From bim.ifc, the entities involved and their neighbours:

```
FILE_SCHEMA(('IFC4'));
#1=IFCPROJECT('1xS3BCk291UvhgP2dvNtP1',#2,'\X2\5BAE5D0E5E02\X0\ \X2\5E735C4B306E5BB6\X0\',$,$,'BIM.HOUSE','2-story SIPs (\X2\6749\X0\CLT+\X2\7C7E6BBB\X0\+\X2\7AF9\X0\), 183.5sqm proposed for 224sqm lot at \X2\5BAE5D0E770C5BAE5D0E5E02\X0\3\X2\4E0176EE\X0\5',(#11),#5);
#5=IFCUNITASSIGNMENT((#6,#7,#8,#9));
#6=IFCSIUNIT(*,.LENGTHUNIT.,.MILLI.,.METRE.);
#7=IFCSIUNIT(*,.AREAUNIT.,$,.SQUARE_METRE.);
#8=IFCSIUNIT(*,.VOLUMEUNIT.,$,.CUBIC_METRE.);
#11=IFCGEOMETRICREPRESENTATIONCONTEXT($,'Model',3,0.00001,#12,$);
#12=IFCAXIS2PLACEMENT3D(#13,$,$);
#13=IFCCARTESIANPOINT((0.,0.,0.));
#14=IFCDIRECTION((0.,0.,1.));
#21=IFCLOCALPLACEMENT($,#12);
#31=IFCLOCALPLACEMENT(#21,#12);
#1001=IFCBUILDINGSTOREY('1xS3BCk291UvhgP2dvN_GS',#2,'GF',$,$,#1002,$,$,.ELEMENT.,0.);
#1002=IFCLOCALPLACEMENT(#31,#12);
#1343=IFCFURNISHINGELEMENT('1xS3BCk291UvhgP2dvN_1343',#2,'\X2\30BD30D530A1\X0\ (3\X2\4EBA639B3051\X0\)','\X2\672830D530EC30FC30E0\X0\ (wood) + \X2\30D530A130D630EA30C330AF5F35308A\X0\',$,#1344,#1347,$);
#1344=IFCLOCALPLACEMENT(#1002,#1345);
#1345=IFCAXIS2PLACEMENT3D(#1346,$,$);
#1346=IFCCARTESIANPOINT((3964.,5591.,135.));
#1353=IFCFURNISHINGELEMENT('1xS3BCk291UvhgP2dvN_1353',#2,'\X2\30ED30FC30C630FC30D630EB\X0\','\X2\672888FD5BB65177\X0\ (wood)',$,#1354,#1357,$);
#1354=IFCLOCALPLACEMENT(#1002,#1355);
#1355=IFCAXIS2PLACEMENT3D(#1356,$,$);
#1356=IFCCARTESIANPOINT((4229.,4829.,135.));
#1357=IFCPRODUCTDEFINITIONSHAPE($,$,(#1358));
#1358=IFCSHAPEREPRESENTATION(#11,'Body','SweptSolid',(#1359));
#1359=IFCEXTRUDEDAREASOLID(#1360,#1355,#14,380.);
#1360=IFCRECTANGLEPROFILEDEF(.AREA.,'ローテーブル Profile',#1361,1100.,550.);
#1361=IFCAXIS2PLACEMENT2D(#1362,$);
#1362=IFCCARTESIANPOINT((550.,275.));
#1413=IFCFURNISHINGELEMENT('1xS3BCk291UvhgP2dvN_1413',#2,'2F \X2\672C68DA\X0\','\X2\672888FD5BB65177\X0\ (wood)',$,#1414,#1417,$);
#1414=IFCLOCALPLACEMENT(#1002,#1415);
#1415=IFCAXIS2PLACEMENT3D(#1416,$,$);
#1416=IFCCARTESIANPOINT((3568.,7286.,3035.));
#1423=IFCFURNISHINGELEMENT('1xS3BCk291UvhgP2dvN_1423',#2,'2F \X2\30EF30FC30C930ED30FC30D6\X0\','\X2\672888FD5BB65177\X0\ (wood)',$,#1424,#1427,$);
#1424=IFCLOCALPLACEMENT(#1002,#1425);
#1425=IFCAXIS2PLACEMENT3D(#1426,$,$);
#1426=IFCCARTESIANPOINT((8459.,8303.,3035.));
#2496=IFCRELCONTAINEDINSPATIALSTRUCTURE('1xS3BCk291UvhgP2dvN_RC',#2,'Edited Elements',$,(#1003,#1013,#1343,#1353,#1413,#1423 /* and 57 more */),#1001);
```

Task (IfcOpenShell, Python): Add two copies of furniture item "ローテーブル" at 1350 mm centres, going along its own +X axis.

```python
import ifcopenshell
import ifcopenshell.api.geometry
import ifcopenshell.api.root
import ifcopenshell.util.element
import ifcopenshell.util.placement
import ifcopenshell.util.unit

model = ifcopenshell.open("bim.ifc")
unit_scale = ifcopenshell.util.unit.calculate_unit_scale(model)


def reuse_history(source, copy):
    """copy_class also copies each property set's owner history, people and application; keep the originals."""
    for rel in copy.IsDefinedBy:
        if rel.is_a("IfcRelDefinesByProperties") and (history := rel.RelatingPropertyDefinition.OwnerHistory):
            rel.RelatingPropertyDefinition.OwnerHistory = source.OwnerHistory
            ifcopenshell.util.element.remove_deep2(model, history)


source = model.by_id(1353)
base = ifcopenshell.util.placement.get_local_placement(source.ObjectPlacement)
step = base[:3, 0] * 1.35 / unit_scale

for i in range(1, 3):
    copy = ifcopenshell.api.root.copy_class(model, product=source)
    copy.Representation = ifcopenshell.util.element.copy_deep(
        model, source.Representation, exclude=["IfcGeometricRepresentationContext", "IfcRepresentationMap"]
    )
    reuse_history(source, copy)
    matrix = base.copy()
    matrix[:3, 3] += i * step
    print("added at", matrix[:3, 3].round(3) + 0.0)
    ifcopenshell.api.geometry.edit_object_placement(model, product=copy, matrix=matrix, is_si=False)

model.write("bim-out.ifc")
```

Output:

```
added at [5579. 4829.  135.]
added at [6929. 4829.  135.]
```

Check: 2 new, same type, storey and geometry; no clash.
